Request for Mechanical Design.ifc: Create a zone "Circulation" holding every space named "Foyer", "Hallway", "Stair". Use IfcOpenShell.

First a look at what the model holds.

```python
import ifcopenshell

model = ifcopenshell.open("Mechanical Design.ifc")
print(model.schema)
seen = {}
for space in model.by_type("IfcSpace"):
    seen[space.LongName] = seen.get(space.LongName, 0) + 1
for name, count in sorted(seen.items(), key=str):
    print(count, "x", name)
print("zones:", [z.Name for z in model.by_type("IfcZone")][:20])
```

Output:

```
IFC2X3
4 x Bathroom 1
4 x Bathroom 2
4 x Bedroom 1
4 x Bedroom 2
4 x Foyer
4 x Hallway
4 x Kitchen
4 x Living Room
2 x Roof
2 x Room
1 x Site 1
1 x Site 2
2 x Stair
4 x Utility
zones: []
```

```python
import ifcopenshell
import ifcopenshell.api.group
import ifcopenshell.api.root

model = ifcopenshell.open("Mechanical Design.ifc")

names = {"Foyer", "Hallway", "Stair"}
spaces = [s for s in model.by_type("IfcSpace") if s.LongName in names]

zone = ifcopenshell.api.root.create_entity(model, ifc_class="IfcZone", name="Circulation")
ifcopenshell.api.group.assign_group(model, products=spaces, group=zone)
print(len(spaces), "spaces in", zone.Name)

model.write("Mechanical Design_v2.ifc")
```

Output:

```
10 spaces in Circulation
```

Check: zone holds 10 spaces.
